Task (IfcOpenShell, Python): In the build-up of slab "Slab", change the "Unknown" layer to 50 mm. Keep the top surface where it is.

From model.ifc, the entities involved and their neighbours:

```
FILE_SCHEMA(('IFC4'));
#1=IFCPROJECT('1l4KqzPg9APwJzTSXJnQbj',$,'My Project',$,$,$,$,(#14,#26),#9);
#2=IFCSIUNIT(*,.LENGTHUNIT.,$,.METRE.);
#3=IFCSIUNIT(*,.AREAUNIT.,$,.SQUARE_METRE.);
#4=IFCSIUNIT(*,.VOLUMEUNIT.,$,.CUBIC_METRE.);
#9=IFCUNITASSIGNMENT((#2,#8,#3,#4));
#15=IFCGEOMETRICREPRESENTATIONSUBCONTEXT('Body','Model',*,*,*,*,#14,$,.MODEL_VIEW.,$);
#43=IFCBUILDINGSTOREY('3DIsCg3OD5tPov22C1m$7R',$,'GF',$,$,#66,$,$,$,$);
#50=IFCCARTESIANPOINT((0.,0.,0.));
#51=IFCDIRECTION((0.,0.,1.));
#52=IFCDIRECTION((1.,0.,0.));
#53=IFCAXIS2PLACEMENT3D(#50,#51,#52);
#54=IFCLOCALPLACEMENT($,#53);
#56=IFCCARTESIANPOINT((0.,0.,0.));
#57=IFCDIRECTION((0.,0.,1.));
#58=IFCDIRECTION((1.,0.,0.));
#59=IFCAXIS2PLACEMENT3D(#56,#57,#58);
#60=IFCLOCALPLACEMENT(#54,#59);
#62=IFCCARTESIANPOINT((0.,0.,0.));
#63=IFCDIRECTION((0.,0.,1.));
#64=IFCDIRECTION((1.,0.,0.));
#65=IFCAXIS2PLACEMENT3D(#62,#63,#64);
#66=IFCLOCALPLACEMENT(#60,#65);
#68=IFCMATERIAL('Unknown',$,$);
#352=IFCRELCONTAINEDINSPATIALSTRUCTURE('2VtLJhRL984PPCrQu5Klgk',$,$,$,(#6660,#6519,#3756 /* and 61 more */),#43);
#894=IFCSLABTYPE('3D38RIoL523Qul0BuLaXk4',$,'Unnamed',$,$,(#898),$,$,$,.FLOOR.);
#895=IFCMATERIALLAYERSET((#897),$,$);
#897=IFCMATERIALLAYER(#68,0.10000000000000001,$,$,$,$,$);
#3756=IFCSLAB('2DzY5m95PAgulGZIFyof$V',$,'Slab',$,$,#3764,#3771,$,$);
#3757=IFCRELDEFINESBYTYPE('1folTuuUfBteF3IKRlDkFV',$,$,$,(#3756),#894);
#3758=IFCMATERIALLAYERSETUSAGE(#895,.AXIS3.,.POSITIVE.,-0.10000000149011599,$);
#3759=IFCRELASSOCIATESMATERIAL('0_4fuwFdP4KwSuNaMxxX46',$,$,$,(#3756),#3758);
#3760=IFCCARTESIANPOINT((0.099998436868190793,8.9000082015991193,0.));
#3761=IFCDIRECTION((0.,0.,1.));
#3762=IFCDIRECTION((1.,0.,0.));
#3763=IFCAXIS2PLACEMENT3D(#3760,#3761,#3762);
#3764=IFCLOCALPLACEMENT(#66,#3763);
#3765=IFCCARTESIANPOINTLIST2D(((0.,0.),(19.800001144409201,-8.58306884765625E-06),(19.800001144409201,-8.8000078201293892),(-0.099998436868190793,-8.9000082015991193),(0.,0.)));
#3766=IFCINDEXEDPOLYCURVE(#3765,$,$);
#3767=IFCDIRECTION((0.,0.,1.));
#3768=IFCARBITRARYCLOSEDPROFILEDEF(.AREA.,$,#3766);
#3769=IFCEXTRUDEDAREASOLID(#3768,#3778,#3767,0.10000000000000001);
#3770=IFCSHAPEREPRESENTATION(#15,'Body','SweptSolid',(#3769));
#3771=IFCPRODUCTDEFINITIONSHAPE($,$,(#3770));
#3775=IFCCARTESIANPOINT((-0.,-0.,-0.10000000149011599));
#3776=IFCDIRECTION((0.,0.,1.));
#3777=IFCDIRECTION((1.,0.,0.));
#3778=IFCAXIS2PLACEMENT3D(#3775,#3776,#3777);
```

```python
import ifcopenshell
import ifcopenshell.util.element
import ifcopenshell.util.representation

model = ifcopenshell.open("model.ifc")

layer_set = model.by_id(895)
layer = next(l for l in layer_set.MaterialLayers if l.Material and l.Material.Name == "Unknown")
change = 0.05 - layer.LayerThickness
layer.LayerThickness += change

# Geometry does not follow the layer set by itself.
slabs = [e for e in ifcopenshell.util.element.get_elements_by_material(model, layer_set) if e.is_a("IfcSlab")]
for slab in sorted(slabs, key=lambda e: e.id()):
    body = ifcopenshell.util.representation.get_representation(slab, "Model", "Body")
    solid = body.Items[0]
    old_depth = solid.Depth
    solid.Depth += change
    # Extruded upwards: lower the start of the extrusion so the top stays.
    x, y, z = solid.Position.Location.Coordinates
    solid.Position.Location = model.createIfcCartesianPoint((x, y, z - change))
    print(slab.id(), f"{old_depth:g} -> {solid.Depth:g}")

# The layers are counted up from the underside, which has moved.
for usage in {ifcopenshell.util.element.get_material(slab) for slab in slabs}:
    usage.OffsetFromReferenceLine -= change

model.write("model_v2.ifc")
```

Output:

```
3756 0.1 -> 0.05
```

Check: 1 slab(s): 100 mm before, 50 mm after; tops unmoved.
